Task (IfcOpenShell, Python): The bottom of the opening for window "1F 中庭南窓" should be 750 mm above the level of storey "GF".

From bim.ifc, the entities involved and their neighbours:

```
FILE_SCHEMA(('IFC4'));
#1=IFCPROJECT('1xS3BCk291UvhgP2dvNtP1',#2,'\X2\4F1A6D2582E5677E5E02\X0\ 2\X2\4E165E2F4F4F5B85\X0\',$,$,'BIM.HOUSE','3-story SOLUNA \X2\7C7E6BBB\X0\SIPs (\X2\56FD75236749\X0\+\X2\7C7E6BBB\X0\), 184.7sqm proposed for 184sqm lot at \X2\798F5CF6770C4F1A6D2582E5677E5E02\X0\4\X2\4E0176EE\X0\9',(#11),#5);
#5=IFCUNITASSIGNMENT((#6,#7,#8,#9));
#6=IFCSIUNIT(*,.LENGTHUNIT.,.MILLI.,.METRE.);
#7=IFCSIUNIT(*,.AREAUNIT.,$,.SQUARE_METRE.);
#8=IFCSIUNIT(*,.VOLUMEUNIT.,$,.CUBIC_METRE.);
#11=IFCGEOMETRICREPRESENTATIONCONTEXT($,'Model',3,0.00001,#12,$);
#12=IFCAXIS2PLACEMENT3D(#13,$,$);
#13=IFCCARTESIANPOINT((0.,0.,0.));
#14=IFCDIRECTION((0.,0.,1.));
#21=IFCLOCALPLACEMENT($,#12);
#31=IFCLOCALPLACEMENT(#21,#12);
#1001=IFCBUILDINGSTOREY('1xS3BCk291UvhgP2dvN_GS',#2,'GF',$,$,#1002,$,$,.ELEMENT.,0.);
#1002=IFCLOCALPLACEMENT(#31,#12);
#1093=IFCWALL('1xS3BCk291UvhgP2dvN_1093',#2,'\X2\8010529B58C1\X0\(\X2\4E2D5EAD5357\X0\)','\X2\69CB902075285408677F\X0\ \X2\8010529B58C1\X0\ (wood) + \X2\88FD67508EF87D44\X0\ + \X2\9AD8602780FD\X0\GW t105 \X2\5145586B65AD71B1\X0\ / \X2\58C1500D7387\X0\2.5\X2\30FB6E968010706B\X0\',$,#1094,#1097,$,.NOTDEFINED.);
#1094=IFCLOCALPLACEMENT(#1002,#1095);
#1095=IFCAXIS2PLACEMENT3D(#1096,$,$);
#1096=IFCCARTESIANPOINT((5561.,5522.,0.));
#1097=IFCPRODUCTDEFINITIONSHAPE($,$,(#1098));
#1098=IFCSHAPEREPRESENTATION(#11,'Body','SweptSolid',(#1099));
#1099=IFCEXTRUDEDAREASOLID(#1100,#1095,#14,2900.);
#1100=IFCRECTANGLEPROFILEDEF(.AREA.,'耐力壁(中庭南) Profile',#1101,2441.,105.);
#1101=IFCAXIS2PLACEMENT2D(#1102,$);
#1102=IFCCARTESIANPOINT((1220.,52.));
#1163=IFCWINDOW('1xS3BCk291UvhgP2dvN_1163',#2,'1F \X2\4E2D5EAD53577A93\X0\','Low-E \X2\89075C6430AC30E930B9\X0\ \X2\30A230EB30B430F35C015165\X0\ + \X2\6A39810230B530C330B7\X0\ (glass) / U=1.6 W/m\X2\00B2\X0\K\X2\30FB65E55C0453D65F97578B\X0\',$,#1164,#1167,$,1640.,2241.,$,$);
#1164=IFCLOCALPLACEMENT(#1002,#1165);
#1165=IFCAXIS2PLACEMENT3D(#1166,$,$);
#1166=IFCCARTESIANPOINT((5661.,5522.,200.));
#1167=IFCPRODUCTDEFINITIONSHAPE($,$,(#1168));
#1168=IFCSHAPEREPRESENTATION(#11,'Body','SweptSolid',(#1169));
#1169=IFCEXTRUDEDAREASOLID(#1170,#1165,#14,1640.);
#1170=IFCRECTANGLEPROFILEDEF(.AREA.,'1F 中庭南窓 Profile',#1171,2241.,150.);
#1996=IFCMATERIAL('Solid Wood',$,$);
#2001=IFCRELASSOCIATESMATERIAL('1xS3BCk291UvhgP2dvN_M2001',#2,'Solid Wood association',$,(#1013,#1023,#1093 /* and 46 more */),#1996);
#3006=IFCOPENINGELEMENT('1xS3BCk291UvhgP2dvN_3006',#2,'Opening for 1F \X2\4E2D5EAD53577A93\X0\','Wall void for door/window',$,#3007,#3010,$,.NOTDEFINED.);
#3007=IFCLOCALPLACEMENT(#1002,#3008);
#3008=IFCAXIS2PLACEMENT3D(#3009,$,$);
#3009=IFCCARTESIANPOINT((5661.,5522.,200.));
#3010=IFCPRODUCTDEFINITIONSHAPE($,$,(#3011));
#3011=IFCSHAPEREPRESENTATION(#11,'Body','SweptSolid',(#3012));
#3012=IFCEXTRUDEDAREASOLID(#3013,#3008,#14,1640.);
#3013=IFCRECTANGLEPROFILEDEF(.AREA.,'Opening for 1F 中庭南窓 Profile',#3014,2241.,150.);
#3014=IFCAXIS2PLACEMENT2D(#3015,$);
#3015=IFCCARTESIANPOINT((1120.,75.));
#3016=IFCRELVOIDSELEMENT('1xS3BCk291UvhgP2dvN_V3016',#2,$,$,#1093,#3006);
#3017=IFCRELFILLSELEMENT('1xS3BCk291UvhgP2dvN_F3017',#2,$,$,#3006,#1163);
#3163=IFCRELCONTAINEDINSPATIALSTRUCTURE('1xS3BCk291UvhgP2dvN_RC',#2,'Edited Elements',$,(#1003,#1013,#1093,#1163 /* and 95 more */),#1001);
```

```python
import numpy as np
import ifcopenshell
import ifcopenshell.api.geometry
import ifcopenshell.geom
import ifcopenshell.util.element
import ifcopenshell.util.placement
import ifcopenshell.util.shape
import ifcopenshell.util.unit

model = ifcopenshell.open("bim.ifc")
unit_scale = ifcopenshell.util.unit.calculate_unit_scale(model)

window = model.by_id(1163)
opening = window.FillsVoids[0].RelatingOpeningElement
storey = ifcopenshell.util.element.get_container(window, ifc_class="IfcBuildingStorey")
level = ifcopenshell.util.placement.get_local_placement(storey.ObjectPlacement)[2, 3]

# The opening's origin need not be at the sill, so measure its lowest point.
shape = ifcopenshell.geom.create_shape(ifcopenshell.geom.settings(), opening)
bottom = ifcopenshell.util.shape.get_shape_bottom_elevation(shape, shape.geometry) / unit_scale
dz = level + 0.75 / unit_scale - bottom

shift = np.array([0.0, 0.0, dz])
# The window is not placed relative to its opening, so move both.
for product in (opening, window):
    matrix = ifcopenshell.util.placement.get_local_placement(product.ObjectPlacement)
    matrix[:3, 3] += shift
    ifcopenshell.api.geometry.edit_object_placement(model, product=product, matrix=matrix, is_si=False)

print(f"moved by {dz * unit_scale:+.3f} m")

model.write("bim_v2.ifc")
```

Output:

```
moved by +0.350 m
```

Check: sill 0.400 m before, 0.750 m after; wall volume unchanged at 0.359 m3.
